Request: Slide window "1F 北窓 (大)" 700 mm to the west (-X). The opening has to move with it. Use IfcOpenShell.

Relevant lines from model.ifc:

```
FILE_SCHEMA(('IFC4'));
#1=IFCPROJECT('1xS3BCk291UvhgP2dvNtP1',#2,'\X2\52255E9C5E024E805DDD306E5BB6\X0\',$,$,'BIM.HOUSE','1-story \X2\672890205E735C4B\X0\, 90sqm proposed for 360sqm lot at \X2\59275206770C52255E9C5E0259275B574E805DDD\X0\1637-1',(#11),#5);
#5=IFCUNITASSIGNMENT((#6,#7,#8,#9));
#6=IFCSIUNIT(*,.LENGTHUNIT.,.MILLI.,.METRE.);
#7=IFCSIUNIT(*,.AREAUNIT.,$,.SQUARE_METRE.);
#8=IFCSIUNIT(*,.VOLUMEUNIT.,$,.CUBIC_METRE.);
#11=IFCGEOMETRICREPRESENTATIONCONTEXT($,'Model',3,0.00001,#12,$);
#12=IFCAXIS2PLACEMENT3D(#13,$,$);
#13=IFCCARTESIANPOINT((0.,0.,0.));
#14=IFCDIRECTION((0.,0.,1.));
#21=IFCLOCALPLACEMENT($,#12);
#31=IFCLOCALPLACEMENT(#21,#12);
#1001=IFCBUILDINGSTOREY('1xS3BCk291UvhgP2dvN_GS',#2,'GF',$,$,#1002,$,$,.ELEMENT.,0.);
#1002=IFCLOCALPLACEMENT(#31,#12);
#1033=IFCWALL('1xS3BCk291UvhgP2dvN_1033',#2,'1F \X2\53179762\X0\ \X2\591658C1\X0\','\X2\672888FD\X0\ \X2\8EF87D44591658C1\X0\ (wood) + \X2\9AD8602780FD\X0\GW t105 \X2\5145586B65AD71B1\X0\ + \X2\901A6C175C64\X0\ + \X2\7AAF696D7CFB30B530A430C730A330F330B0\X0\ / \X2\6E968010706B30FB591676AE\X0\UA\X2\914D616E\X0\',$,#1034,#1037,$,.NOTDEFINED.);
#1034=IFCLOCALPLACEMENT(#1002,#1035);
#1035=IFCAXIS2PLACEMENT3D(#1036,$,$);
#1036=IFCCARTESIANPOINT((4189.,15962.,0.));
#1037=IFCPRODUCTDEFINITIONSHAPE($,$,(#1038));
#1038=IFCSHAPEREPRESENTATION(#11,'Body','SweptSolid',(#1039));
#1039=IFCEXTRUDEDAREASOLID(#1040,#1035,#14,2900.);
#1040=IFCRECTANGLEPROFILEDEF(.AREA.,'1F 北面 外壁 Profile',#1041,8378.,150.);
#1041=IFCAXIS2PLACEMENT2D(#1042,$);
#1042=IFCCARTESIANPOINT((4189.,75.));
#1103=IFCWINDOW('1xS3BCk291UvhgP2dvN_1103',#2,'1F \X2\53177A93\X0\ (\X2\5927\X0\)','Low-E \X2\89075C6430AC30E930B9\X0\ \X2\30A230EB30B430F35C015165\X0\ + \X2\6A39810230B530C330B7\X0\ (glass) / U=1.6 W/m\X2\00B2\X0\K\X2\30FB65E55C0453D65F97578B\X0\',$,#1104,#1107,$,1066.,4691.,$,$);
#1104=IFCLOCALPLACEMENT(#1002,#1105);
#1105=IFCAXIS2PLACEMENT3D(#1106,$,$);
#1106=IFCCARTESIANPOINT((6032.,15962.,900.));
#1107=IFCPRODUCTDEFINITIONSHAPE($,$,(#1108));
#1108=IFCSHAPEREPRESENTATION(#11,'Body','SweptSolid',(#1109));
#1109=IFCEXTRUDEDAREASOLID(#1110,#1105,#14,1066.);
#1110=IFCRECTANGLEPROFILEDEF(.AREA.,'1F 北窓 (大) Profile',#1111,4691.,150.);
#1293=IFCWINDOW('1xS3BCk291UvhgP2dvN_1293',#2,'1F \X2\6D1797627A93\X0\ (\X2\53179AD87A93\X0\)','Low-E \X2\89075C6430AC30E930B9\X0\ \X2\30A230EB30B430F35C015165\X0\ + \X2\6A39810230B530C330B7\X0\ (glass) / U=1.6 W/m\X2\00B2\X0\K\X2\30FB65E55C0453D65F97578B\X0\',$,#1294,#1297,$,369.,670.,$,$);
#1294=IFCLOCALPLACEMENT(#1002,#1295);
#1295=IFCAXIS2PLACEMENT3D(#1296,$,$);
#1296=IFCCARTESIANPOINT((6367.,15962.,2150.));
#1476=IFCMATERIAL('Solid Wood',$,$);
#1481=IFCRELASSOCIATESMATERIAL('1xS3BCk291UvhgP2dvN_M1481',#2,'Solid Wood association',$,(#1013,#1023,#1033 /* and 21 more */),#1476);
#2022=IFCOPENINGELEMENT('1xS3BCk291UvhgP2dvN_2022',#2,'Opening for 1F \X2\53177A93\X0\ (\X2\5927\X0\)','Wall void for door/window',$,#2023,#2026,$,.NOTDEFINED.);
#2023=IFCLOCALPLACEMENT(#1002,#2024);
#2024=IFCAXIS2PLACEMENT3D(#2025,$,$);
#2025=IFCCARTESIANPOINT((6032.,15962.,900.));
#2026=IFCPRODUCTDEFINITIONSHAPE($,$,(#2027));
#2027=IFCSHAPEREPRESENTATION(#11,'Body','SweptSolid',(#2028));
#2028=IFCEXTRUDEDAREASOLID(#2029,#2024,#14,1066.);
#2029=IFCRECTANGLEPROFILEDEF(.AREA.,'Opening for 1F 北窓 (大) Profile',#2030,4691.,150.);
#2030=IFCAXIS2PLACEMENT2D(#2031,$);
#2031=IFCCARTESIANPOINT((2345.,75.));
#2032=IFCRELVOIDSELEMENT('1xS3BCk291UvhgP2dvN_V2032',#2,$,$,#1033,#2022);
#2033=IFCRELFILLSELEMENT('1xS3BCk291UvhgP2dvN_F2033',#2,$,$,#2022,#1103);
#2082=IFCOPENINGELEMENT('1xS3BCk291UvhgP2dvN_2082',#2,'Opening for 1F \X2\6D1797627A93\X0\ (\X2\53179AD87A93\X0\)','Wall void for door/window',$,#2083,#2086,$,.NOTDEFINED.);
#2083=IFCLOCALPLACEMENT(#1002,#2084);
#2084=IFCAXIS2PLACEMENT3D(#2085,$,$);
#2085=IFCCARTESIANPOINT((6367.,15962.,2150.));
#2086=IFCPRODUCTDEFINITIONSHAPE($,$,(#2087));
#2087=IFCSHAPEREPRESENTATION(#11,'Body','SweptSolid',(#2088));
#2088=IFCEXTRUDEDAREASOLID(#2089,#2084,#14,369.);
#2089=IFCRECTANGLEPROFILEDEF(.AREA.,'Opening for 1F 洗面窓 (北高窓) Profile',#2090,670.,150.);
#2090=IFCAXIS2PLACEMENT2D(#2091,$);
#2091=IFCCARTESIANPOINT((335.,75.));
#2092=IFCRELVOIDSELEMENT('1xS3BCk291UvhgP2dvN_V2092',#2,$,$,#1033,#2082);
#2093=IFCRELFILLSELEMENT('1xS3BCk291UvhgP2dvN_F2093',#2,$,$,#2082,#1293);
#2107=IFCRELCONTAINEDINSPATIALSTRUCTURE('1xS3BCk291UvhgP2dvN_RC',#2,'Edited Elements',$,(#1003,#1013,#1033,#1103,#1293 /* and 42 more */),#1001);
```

```python
import ifcopenshell
import ifcopenshell.api.geometry
import ifcopenshell.util.placement
import ifcopenshell.util.unit

model = ifcopenshell.open("model.ifc")
unit_scale = ifcopenshell.util.unit.calculate_unit_scale(model)

window = model.by_id(1103)
opening = window.FillsVoids[0].RelatingOpeningElement
wall = opening.VoidsElements[0].RelatingBuildingElement

wall_matrix = ifcopenshell.util.placement.get_local_placement(wall.ObjectPlacement)
shift = wall_matrix[:3, 0] * -0.7 / unit_scale
before = ifcopenshell.util.placement.get_local_placement(window.ObjectPlacement)[:3, 3].copy()

# The window is not placed relative to its opening, so move both.
for product in (opening, window):
    matrix = ifcopenshell.util.placement.get_local_placement(product.ObjectPlacement)
    matrix[:3, 3] += shift
    ifcopenshell.api.geometry.edit_object_placement(model, product=product, matrix=matrix, is_si=False)

after = ifcopenshell.util.placement.get_local_placement(window.ObjectPlacement)[:3, 3]
print("window moved by", (after - before).round(3) + 0.0)

model.write("model_updated.ifc")
```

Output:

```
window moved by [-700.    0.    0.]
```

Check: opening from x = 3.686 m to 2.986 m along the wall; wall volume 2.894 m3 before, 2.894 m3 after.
